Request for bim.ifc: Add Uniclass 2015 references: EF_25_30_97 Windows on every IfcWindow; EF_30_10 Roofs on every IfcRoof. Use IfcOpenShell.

First a look at what the model holds.

```python
import ifcopenshell

model = ifcopenshell.open("bim.ifc")
print(model.schema)
print("classifications:", [c.Name for c in model.by_type("IfcClassification")])
for ifc_class in ("IfcDoor", "IfcRoof", "IfcStair", "IfcWall", "IfcWindow"):
    print(ifc_class, len(model.by_type(ifc_class)))
```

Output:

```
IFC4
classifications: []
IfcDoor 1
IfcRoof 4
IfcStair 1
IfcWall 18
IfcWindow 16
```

```python
import ifcopenshell
import ifcopenshell.api.classification

model = ifcopenshell.open("bim.ifc")

system = ifcopenshell.api.classification.add_classification(model, classification="Uniclass 2015")

codes = {
    "IfcWindow": ("EF_25_30_97", "Windows"),
    "IfcRoof": ("EF_30_10", "Roofs"),
}
for ifc_class, (code, name) in codes.items():
    products = model.by_type(ifc_class)
    ifcopenshell.api.classification.add_reference(
        model, products=products, classification=system, identification=code, name=name
    )
    print(code, len(products))

model.write("bim_v2.ifc")
```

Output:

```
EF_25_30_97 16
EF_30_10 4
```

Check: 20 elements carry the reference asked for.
